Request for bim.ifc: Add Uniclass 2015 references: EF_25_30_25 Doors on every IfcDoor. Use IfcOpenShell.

First a look at what the model holds.

```python
import ifcopenshell

model = ifcopenshell.open("bim.ifc")
print(model.schema)
print("classifications:", [c.Name for c in model.by_type("IfcClassification")])
for ifc_class in ("IfcDoor", "IfcRoof", "IfcStair", "IfcWall", "IfcWindow"):
    print(ifc_class, len(model.by_type(ifc_class)))
```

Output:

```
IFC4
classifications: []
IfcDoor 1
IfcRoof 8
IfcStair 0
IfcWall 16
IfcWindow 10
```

```python
import ifcopenshell
import ifcopenshell.api.classification

model = ifcopenshell.open("bim.ifc")

system = ifcopenshell.api.classification.add_classification(model, classification="Uniclass 2015")

codes = {
    "IfcDoor": ("EF_25_30_25", "Doors"),
}
for ifc_class, (code, name) in codes.items():
    products = model.by_type(ifc_class)
    ifcopenshell.api.classification.add_reference(
        model, products=products, classification=system, identification=code, name=name
    )
    print(code, len(products))

model.write("bim_rev.ifc")
```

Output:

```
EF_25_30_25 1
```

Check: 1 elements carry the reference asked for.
